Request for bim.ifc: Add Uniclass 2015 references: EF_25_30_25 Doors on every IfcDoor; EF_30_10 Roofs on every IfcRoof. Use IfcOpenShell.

First a look at what the model holds.

```python
import ifcopenshell

model = ifcopenshell.open("bim.ifc")
print(model.schema)
print("classifications:", [c.Name for c in model.by_type("IfcClassification")])
for ifc_class in ("IfcDoor", "IfcRoof", "IfcStair", "IfcWall", "IfcWindow"):
    print(ifc_class, len(model.by_type(ifc_class)))
```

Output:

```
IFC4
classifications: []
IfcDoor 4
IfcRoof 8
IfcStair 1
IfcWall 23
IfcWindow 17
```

```python
import ifcopenshell
import ifcopenshell.api.classification

model = ifcopenshell.open("bim.ifc")

system = ifcopenshell.api.classification.add_classification(model, classification="Uniclass 2015")

codes = {
    "IfcDoor": ("EF_25_30_25", "Doors"),
    "IfcRoof": ("EF_30_10", "Roofs"),
}
for ifc_class, (code, name) in codes.items():
    products = model.by_type(ifc_class)
    ifcopenshell.api.classification.add_reference(
        model, products=products, classification=system, identification=code, name=name
    )
    print(code, len(products))

model.write("bim-out.ifc")
```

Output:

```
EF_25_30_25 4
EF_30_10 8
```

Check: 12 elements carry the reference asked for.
